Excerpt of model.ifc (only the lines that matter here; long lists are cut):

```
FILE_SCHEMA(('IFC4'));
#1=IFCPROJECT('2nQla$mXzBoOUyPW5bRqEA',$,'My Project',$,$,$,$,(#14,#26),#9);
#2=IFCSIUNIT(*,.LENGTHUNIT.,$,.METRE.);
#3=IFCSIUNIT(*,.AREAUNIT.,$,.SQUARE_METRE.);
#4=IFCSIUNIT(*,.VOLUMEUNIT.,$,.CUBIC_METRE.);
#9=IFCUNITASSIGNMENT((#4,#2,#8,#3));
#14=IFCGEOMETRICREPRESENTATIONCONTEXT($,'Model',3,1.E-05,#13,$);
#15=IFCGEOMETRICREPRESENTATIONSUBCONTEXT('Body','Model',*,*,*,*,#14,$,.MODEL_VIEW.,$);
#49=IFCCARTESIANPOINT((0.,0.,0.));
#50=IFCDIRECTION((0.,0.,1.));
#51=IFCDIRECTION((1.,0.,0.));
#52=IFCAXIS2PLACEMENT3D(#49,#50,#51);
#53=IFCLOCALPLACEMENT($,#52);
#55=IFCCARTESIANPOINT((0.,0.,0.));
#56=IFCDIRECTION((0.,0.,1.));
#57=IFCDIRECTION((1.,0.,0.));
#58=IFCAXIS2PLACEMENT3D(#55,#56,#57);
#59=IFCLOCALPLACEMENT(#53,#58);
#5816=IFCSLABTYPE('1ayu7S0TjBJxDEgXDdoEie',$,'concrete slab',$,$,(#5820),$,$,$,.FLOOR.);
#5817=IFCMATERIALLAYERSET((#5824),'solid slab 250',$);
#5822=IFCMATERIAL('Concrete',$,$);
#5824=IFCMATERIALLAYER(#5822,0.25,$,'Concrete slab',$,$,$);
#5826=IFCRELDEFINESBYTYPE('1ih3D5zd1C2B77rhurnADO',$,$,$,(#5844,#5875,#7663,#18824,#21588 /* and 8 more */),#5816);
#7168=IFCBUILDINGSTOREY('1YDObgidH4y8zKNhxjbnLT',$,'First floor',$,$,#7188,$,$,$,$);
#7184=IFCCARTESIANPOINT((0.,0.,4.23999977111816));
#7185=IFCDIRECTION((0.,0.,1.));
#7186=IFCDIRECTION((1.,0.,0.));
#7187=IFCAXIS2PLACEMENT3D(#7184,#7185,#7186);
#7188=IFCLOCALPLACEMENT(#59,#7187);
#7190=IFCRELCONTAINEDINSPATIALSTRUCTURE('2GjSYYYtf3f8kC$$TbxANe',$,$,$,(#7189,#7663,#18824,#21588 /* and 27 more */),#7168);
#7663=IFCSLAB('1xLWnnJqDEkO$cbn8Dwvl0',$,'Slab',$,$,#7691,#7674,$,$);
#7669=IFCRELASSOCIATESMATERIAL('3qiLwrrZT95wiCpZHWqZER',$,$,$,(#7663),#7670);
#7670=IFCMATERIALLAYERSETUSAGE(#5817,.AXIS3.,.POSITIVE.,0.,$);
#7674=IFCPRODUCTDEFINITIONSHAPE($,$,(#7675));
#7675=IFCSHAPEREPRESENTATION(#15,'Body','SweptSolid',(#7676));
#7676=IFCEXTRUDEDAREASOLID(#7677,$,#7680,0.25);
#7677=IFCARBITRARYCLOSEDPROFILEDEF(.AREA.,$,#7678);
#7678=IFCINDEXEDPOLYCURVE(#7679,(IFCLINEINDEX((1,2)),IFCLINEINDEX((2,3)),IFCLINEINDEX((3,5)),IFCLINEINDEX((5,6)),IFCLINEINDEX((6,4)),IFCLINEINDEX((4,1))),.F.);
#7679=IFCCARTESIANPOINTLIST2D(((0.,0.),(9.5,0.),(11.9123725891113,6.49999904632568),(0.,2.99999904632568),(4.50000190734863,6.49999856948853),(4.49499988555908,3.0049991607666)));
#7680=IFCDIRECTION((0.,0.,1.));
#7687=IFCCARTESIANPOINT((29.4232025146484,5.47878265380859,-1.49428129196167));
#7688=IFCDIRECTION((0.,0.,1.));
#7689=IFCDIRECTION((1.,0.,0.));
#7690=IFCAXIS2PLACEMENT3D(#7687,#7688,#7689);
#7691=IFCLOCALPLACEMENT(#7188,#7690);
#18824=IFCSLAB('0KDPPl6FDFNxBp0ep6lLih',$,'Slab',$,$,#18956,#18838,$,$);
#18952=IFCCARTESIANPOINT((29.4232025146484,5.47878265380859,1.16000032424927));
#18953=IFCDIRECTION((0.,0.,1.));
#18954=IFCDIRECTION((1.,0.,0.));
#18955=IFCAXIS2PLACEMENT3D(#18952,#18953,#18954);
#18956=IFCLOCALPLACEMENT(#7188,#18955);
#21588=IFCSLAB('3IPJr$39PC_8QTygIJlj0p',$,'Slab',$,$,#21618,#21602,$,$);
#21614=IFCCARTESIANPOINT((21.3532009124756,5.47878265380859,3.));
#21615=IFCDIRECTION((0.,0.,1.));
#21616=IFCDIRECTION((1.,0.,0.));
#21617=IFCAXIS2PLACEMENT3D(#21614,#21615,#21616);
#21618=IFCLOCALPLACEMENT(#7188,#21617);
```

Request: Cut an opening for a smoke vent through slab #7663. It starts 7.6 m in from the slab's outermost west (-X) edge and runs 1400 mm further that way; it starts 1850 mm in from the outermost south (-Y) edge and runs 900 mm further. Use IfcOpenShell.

```python
import numpy as np
import ifcopenshell
import ifcopenshell.api.feature
import ifcopenshell.api.geometry
import ifcopenshell.api.root
import ifcopenshell.geom
import ifcopenshell.util.placement
import ifcopenshell.util.representation
import ifcopenshell.util.shape
import ifcopenshell.util.unit

model = ifcopenshell.open("model.ifc")
unit_scale = ifcopenshell.util.unit.calculate_unit_scale(model)
settings = ifcopenshell.geom.settings()


def volume(element):
    """Net volume in cubic metres, openings subtracted."""
    shape = ifcopenshell.geom.create_shape(settings, element)
    return ifcopenshell.util.shape.get_volume(shape.geometry)


slab = model.by_guid("1xLWnnJqDEkO$cbn8Dwvl0")
before = volume(slab)

# Extent in the slab's own axes, in metres. The edges named are its -X and -Y sides.
slab_shape = ifcopenshell.geom.create_shape(settings, slab)
vertices = ifcopenshell.util.shape.get_vertices(slab_shape.geometry)
x_min, y_min, bottom = vertices.min(axis=0)
top = vertices[:, 2].max()

opening = ifcopenshell.api.root.create_entity(model, ifc_class="IfcOpeningElement", name="Smoke vent opening", predefined_type="OPENING")
context = ifcopenshell.util.representation.get_context(model, "Model", "Body", "MODEL_VIEW")
width, depth = 1.4, 0.9
outline = [(0.0, 0.0), (width, 0.0), (width, depth), (0.0, depth), (0.0, 0.0)]
# Overshoot both faces by 50 mm so the cut is clean.
shape = ifcopenshell.api.geometry.add_slab_representation(
    model, context=context, depth=top - bottom + 0.1, polyline=outline
)
ifcopenshell.api.geometry.assign_representation(model, product=opening, representation=shape)

matrix = ifcopenshell.util.placement.get_local_placement(slab.ObjectPlacement)
matrix[:, 3] = matrix @ np.append(np.array([x_min + 7.6, y_min + 1.85, bottom - 0.05]) / unit_scale, 1.0)
ifcopenshell.api.geometry.edit_object_placement(model, product=opening, matrix=matrix, is_si=False)
ifcopenshell.api.feature.add_feature(model, feature=opening, element=slab)

after = volume(slab)

print(f"slab volume {before:.3f} -> {after:.3f} m3")

model.write("model-out.ifc")
```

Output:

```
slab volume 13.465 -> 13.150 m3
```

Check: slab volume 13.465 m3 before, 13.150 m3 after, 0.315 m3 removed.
